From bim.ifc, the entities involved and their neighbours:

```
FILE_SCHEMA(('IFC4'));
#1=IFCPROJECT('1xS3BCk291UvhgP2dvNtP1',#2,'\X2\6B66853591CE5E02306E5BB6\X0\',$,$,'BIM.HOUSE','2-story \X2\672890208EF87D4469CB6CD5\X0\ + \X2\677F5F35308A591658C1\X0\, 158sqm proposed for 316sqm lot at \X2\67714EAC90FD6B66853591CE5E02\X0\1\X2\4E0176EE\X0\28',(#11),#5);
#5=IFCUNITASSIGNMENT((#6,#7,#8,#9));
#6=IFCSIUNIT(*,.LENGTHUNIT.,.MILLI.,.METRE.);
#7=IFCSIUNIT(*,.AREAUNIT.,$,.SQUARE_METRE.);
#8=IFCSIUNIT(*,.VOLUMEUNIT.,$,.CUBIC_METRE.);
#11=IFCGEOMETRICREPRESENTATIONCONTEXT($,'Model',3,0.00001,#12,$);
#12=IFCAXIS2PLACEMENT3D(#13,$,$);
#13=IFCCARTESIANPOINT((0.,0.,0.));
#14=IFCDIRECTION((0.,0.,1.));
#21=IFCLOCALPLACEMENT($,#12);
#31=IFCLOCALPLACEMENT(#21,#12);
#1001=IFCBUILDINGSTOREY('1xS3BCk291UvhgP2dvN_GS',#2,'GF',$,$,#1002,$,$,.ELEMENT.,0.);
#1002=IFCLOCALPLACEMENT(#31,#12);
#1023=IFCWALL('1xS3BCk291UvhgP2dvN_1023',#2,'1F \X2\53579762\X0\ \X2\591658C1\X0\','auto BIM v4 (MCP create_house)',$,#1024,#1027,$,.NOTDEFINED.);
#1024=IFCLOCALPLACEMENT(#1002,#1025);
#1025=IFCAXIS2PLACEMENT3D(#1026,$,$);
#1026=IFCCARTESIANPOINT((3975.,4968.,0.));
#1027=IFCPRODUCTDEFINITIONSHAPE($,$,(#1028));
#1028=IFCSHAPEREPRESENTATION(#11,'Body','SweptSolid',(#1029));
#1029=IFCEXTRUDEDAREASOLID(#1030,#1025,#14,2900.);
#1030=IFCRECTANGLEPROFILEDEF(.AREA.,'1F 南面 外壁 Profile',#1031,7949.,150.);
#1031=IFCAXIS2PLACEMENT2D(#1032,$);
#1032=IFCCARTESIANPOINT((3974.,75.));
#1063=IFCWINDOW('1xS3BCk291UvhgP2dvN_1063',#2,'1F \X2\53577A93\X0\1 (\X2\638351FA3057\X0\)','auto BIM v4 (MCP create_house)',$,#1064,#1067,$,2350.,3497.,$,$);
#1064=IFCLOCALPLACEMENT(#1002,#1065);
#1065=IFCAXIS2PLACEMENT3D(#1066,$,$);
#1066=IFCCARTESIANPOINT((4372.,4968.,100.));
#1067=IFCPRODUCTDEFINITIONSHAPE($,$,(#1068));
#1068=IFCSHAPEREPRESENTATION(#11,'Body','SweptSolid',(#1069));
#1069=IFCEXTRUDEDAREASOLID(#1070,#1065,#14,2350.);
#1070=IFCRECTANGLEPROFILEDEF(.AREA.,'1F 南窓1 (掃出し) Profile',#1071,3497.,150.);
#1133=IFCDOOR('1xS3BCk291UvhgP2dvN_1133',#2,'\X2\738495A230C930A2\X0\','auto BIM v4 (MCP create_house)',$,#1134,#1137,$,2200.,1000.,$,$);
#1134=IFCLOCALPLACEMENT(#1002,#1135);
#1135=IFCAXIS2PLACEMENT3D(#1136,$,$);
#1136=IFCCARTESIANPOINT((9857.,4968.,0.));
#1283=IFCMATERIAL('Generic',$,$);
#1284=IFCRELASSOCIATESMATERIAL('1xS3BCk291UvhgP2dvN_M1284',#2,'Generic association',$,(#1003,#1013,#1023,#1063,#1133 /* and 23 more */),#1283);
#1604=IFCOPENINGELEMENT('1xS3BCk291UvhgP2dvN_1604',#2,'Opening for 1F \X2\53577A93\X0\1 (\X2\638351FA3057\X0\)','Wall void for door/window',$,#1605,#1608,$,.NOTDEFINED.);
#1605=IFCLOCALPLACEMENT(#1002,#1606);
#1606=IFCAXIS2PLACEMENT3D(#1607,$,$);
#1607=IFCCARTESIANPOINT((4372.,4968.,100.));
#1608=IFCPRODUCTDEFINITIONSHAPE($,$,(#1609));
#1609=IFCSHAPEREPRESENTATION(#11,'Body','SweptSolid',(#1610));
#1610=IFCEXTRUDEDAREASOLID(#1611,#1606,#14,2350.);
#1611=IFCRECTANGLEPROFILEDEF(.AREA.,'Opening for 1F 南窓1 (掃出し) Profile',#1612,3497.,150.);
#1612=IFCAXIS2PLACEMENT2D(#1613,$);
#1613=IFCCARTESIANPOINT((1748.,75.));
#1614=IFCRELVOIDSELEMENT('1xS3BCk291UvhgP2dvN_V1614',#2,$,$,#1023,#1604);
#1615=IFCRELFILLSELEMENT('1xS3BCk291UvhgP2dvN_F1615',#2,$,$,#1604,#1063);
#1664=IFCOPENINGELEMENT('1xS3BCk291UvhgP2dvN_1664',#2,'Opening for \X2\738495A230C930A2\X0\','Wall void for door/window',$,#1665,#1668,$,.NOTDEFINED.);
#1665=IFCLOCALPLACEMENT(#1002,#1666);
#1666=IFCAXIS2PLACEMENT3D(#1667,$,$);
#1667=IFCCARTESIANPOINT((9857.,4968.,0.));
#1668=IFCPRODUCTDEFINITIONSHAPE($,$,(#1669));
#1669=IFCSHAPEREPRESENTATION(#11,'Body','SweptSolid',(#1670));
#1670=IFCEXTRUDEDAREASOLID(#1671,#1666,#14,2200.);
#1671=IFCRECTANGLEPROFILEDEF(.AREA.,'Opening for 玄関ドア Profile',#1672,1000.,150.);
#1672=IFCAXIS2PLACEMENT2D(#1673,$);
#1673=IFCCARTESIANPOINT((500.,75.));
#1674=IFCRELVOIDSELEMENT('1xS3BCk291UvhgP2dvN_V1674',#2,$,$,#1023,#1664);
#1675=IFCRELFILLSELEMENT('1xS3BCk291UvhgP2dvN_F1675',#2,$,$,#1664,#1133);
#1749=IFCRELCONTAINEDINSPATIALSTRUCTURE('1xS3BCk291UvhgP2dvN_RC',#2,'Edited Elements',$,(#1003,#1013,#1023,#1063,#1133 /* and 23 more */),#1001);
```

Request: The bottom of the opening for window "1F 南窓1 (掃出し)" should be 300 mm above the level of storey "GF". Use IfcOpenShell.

```python
import numpy as np
import ifcopenshell
import ifcopenshell.api.geometry
import ifcopenshell.geom
import ifcopenshell.util.element
import ifcopenshell.util.placement
import ifcopenshell.util.shape
import ifcopenshell.util.unit

model = ifcopenshell.open("bim.ifc")
unit_scale = ifcopenshell.util.unit.calculate_unit_scale(model)

window = model.by_id(1063)
opening = window.FillsVoids[0].RelatingOpeningElement
storey = ifcopenshell.util.element.get_container(window, ifc_class="IfcBuildingStorey")
level = ifcopenshell.util.placement.get_local_placement(storey.ObjectPlacement)[2, 3]

# The opening's origin need not be at the sill, so measure its lowest point.
shape = ifcopenshell.geom.create_shape(ifcopenshell.geom.settings(), opening)
bottom = ifcopenshell.util.shape.get_shape_bottom_elevation(shape, shape.geometry) / unit_scale
dz = level + 0.3 / unit_scale - bottom

shift = np.array([0.0, 0.0, dz])
# The window is not placed relative to its opening, so move both.
for product in (opening, window):
    matrix = ifcopenshell.util.placement.get_local_placement(product.ObjectPlacement)
    matrix[:3, 3] += shift
    ifcopenshell.api.geometry.edit_object_placement(model, product=product, matrix=matrix, is_si=False)

print(f"moved by {dz * unit_scale:+.3f} m")

model.write("bim_v2.ifc")
```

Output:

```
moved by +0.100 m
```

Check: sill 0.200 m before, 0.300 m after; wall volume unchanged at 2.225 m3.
